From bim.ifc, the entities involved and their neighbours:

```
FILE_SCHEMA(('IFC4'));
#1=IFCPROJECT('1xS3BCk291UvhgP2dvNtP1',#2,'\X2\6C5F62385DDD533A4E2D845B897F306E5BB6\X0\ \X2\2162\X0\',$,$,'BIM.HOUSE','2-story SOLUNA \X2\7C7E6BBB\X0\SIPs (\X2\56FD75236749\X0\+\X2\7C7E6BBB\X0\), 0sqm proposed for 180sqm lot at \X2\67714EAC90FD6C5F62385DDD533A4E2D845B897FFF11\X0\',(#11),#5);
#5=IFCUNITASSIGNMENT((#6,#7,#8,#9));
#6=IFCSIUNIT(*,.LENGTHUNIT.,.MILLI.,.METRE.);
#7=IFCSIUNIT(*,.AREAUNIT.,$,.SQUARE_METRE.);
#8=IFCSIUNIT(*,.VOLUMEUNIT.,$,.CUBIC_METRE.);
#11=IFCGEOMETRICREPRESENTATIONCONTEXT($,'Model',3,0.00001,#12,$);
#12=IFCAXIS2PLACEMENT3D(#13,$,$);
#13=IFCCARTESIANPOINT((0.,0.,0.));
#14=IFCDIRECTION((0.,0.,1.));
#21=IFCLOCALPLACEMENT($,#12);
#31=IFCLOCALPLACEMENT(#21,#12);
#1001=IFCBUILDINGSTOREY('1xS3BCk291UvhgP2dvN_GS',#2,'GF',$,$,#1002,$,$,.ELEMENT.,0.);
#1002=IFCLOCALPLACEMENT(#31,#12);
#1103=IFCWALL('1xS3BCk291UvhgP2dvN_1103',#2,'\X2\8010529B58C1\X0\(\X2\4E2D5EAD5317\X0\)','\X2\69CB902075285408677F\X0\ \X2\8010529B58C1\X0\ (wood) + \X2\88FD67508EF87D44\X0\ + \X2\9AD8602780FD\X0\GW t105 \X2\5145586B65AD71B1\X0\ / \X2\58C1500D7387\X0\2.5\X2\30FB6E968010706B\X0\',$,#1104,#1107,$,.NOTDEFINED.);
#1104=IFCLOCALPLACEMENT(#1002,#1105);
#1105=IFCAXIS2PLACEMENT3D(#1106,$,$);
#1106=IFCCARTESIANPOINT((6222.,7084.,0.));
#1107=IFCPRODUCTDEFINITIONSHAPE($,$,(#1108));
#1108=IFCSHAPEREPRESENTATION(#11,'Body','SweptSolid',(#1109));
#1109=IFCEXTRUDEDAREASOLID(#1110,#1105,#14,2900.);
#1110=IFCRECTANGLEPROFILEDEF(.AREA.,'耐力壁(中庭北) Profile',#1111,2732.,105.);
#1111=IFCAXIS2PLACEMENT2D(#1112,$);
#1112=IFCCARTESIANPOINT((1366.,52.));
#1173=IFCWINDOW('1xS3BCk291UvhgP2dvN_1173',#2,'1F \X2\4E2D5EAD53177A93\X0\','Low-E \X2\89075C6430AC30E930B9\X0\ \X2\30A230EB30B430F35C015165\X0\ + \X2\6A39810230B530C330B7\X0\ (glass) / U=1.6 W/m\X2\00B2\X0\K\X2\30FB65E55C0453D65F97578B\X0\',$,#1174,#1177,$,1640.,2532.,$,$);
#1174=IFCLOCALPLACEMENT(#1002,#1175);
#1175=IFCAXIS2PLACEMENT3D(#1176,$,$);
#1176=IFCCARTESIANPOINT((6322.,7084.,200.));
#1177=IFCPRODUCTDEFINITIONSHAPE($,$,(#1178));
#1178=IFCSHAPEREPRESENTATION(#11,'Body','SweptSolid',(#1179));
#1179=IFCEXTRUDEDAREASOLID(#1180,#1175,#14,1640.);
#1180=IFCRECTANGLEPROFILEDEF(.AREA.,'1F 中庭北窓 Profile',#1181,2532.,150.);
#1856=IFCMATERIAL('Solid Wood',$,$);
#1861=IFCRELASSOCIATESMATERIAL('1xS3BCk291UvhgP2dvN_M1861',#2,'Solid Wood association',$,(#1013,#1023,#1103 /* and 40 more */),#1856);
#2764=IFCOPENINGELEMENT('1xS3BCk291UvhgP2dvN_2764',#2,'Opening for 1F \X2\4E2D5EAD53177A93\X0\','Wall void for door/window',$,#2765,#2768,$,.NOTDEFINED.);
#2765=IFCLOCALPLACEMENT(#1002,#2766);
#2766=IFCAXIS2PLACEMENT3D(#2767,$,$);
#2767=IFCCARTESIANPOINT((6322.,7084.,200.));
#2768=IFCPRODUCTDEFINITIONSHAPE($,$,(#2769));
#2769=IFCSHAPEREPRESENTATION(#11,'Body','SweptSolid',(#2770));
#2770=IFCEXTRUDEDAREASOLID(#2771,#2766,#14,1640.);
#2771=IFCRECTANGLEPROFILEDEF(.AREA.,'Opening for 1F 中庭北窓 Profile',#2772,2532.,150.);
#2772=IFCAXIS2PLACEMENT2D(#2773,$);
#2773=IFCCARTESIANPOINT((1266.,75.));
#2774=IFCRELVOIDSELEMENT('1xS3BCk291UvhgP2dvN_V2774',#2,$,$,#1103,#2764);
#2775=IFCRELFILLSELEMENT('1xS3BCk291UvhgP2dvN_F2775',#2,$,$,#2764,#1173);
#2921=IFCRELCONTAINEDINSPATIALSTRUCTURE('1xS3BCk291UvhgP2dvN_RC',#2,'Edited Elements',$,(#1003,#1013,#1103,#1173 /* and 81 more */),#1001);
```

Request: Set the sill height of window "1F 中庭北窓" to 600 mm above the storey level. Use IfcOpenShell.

```python
import numpy as np
import ifcopenshell
import ifcopenshell.api.geometry
import ifcopenshell.geom
import ifcopenshell.util.element
import ifcopenshell.util.placement
import ifcopenshell.util.shape
import ifcopenshell.util.unit

model = ifcopenshell.open("bim.ifc")
unit_scale = ifcopenshell.util.unit.calculate_unit_scale(model)

window = model.by_guid("1xS3BCk291UvhgP2dvN_1173")
opening = window.FillsVoids[0].RelatingOpeningElement
storey = ifcopenshell.util.element.get_container(window, ifc_class="IfcBuildingStorey")
level = ifcopenshell.util.placement.get_local_placement(storey.ObjectPlacement)[2, 3]

# The opening's origin need not be at the sill, so measure its lowest point.
shape = ifcopenshell.geom.create_shape(ifcopenshell.geom.settings(), opening)
bottom = ifcopenshell.util.shape.get_shape_bottom_elevation(shape, shape.geometry) / unit_scale
dz = level + 0.6 / unit_scale - bottom

shift = np.array([0.0, 0.0, dz])
# The window is not placed relative to its opening, so move both.
for product in (opening, window):
    matrix = ifcopenshell.util.placement.get_local_placement(product.ObjectPlacement)
    matrix[:3, 3] += shift
    ifcopenshell.api.geometry.edit_object_placement(model, product=product, matrix=matrix, is_si=False)

print(f"moved by {dz * unit_scale:+.3f} m")

model.write("bim_rev.ifc")
```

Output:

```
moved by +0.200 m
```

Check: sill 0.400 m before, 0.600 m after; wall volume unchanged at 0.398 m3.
